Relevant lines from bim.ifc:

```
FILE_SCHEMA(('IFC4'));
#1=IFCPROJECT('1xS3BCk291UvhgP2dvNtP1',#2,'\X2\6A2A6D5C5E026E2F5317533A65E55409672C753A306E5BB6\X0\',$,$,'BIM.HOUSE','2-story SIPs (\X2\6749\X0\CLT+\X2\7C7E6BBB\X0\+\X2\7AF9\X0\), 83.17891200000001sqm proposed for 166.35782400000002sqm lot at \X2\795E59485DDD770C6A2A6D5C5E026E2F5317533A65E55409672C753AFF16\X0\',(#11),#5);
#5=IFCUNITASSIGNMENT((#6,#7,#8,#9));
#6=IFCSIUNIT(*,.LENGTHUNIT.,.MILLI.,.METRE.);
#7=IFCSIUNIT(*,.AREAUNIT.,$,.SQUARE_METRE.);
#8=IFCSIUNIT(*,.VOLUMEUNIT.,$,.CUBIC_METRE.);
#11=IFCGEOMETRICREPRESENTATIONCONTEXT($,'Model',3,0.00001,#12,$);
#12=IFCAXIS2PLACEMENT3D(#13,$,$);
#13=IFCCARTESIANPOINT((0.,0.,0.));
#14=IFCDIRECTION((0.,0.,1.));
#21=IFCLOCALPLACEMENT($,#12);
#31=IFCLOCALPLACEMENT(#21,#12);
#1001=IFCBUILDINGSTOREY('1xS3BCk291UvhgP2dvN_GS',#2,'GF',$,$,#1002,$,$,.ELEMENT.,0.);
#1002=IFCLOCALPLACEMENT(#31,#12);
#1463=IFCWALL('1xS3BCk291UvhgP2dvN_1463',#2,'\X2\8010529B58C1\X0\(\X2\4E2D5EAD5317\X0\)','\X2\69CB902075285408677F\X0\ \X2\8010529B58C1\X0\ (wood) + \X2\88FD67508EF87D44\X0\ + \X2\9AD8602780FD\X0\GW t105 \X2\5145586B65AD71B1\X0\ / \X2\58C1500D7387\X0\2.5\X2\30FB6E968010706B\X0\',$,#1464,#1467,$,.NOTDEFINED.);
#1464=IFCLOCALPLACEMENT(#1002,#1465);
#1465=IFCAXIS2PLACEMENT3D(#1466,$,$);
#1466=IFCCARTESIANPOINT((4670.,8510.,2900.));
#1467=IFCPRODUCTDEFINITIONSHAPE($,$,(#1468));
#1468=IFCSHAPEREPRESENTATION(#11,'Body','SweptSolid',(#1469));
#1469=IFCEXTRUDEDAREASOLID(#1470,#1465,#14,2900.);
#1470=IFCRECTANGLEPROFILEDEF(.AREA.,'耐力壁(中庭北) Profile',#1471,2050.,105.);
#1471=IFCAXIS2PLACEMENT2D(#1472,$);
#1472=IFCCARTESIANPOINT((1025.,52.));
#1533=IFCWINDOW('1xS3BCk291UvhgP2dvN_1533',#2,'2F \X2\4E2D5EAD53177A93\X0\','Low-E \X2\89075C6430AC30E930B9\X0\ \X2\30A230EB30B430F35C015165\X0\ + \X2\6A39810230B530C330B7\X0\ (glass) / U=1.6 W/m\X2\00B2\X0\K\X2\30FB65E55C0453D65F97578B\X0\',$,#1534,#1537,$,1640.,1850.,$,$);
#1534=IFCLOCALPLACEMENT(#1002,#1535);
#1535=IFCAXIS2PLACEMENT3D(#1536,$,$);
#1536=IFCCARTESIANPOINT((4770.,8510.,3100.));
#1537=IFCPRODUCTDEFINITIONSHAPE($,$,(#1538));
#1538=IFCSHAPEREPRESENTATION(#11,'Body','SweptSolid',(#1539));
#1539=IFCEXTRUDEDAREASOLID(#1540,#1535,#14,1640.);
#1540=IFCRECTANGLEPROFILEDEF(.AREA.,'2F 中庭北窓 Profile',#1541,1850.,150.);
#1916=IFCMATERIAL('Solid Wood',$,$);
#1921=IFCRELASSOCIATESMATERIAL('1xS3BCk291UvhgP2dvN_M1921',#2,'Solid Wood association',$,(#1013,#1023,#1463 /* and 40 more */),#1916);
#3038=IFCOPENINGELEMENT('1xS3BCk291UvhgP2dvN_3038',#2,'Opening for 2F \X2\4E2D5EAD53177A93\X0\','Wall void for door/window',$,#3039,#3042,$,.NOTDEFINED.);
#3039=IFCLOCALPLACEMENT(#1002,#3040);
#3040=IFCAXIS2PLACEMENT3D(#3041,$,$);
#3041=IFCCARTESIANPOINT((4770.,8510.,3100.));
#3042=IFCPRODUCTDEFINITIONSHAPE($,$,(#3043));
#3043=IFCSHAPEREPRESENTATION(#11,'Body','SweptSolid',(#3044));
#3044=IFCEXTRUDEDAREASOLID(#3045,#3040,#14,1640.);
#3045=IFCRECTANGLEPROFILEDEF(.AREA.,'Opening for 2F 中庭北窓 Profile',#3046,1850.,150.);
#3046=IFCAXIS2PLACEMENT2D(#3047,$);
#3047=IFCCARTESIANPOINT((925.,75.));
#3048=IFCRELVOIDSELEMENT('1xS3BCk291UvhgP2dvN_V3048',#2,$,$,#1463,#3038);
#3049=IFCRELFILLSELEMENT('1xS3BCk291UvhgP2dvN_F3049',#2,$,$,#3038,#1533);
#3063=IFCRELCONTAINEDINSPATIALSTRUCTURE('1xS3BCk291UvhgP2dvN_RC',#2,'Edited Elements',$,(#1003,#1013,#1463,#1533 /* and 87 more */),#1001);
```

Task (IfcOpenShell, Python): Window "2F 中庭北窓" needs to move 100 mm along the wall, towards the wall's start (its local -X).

```python
import ifcopenshell
import ifcopenshell.api.geometry
import ifcopenshell.util.placement

model = ifcopenshell.open("bim.ifc")

window = model.by_guid("1xS3BCk291UvhgP2dvN_1533")
opening = window.FillsVoids[0].RelatingOpeningElement
wall = opening.VoidsElements[0].RelatingBuildingElement

wall_matrix = ifcopenshell.util.placement.get_local_placement(wall.ObjectPlacement)
shift = wall_matrix[:3, 0] * -100.0
before = ifcopenshell.util.placement.get_local_placement(window.ObjectPlacement)[:3, 3].copy()

# The window is not placed relative to its opening, so move both.
for product in (opening, window):
    matrix = ifcopenshell.util.placement.get_local_placement(product.ObjectPlacement)
    matrix[:3, 3] += shift
    ifcopenshell.api.geometry.edit_object_placement(model, product=product, matrix=matrix, is_si=False)

after = ifcopenshell.util.placement.get_local_placement(window.ObjectPlacement)[:3, 3]
print("window moved by", (after - before).round(3) + 0.0)

model.write("bim_rev.ifc")
```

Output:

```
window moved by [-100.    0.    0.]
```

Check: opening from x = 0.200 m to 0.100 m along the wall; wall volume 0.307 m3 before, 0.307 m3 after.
